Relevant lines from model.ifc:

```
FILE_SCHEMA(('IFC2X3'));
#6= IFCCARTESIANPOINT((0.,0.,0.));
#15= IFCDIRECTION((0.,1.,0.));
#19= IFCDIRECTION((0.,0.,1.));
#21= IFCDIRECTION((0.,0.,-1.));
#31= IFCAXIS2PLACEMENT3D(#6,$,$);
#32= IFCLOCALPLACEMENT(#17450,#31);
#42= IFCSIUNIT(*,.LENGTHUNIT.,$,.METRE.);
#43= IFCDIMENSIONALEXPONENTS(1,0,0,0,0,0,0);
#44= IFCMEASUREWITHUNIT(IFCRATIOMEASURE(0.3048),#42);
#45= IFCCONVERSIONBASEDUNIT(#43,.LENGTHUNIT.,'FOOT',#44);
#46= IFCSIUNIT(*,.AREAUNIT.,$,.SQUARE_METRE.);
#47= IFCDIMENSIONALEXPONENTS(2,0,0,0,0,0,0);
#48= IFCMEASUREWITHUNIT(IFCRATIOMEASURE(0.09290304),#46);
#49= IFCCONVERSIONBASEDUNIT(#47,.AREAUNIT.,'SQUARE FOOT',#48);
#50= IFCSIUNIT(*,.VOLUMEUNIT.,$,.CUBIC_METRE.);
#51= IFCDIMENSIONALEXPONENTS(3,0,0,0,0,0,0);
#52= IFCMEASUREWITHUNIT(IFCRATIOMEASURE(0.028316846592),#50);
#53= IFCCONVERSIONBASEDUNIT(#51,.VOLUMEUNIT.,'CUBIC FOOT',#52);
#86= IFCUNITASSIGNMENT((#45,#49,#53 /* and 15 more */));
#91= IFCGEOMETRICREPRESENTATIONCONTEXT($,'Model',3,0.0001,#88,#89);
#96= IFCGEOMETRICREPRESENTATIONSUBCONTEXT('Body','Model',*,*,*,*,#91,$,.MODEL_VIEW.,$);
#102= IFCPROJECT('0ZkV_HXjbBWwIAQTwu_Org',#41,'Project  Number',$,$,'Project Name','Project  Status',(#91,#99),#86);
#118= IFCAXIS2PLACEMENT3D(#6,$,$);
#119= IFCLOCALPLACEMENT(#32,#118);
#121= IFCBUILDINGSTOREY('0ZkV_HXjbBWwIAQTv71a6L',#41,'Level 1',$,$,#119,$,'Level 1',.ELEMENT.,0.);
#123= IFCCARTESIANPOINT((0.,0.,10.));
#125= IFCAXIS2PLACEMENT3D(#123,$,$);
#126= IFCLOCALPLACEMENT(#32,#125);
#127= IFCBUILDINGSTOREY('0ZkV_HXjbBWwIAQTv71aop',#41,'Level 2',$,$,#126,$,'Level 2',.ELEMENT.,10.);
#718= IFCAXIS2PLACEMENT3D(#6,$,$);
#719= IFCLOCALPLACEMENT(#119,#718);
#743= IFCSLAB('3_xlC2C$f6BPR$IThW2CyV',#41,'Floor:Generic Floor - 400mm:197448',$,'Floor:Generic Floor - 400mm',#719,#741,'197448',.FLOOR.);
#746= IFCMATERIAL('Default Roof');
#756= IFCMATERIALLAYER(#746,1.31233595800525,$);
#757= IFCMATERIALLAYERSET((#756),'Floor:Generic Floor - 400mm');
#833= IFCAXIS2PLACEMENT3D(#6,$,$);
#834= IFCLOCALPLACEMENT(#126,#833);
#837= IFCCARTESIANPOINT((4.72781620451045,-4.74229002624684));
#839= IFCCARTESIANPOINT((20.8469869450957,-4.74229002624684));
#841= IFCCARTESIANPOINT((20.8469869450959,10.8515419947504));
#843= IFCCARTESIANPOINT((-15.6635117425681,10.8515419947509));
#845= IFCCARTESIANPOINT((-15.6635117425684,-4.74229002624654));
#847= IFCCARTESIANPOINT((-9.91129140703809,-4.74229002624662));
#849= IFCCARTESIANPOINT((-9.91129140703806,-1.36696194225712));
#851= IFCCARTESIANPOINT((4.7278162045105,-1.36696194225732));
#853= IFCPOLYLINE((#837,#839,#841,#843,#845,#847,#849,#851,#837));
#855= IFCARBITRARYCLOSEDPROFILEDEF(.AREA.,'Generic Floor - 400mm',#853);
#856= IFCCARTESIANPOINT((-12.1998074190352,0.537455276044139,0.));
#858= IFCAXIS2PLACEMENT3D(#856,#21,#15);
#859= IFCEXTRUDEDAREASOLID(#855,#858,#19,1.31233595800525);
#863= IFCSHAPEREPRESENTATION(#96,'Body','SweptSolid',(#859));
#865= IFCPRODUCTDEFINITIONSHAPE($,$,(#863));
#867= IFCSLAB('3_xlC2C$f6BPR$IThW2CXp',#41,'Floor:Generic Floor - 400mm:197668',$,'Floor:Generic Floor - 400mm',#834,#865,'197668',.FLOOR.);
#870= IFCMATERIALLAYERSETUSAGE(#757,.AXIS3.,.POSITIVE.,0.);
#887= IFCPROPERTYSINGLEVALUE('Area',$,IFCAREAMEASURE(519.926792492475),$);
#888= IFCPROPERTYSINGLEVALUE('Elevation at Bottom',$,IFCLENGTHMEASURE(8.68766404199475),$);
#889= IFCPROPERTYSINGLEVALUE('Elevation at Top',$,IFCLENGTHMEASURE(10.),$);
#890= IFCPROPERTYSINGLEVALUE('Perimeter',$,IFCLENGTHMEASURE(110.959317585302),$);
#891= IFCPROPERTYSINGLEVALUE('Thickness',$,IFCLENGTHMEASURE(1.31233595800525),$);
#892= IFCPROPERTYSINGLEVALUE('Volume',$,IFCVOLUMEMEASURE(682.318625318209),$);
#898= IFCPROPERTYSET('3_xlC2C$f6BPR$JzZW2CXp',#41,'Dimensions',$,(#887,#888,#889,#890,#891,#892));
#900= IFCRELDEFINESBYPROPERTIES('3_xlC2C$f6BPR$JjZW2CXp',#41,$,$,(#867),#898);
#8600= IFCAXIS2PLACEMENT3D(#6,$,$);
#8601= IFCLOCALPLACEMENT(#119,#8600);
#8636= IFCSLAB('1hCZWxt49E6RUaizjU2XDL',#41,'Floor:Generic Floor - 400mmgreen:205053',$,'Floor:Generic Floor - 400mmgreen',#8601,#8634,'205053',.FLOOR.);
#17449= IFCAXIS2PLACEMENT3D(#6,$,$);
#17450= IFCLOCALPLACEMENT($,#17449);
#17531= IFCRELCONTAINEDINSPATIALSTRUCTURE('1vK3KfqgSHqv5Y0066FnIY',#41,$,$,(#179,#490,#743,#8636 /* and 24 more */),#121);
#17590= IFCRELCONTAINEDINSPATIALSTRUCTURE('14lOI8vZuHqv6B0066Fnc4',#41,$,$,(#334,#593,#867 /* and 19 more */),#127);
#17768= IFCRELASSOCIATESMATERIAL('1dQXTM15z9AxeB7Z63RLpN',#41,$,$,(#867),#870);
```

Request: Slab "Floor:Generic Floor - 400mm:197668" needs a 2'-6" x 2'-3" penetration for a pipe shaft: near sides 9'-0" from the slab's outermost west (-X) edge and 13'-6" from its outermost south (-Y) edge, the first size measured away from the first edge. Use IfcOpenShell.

```python
import numpy as np
import ifcopenshell
import ifcopenshell.api.feature
import ifcopenshell.api.geometry
import ifcopenshell.api.pset
import ifcopenshell.api.root
import ifcopenshell.geom
import ifcopenshell.util.element
import ifcopenshell.util.placement
import ifcopenshell.util.representation
import ifcopenshell.util.shape
import ifcopenshell.util.unit

model = ifcopenshell.open("model.ifc")
unit_scale = ifcopenshell.util.unit.calculate_unit_scale(model)
area_scale = ifcopenshell.util.unit.calculate_unit_scale(model, "AREAUNIT")
volume_scale = ifcopenshell.util.unit.calculate_unit_scale(model, "VOLUMEUNIT")
settings = ifcopenshell.geom.settings()


def volume(element):
    """Net volume in cubic metres, openings subtracted."""
    shape = ifcopenshell.geom.create_shape(settings, element)
    return ifcopenshell.util.shape.get_volume(shape.geometry)


slab = model.by_id(867)
before = volume(slab)

# Extent in the slab's own axes, in metres. The edges named are its -X and -Y sides.
slab_shape = ifcopenshell.geom.create_shape(settings, slab)
vertices = ifcopenshell.util.shape.get_vertices(slab_shape.geometry)
x_min, y_min, bottom = vertices.min(axis=0)
top = vertices[:, 2].max()

opening = ifcopenshell.api.root.create_entity(model, ifc_class="IfcOpeningElement", name="Pipe shaft opening")
context = ifcopenshell.util.representation.get_context(model, "Model", "Body", "MODEL_VIEW")
width, depth = 0.762, 0.6858
outline = [(0.0, 0.0), (width, 0.0), (width, depth), (0.0, depth), (0.0, 0.0)]
# Overshoot both faces by 50 mm so the cut is clean.
shape = ifcopenshell.api.geometry.add_slab_representation(
    model, context=context, depth=top - bottom + 0.1, polyline=outline
)
ifcopenshell.api.geometry.assign_representation(model, product=opening, representation=shape)

matrix = ifcopenshell.util.placement.get_local_placement(slab.ObjectPlacement)
matrix[:, 3] = matrix @ np.append(np.array([x_min + 2.7432, y_min + 4.1148, bottom - 0.05]) / unit_scale, 1.0)
ifcopenshell.api.geometry.edit_object_placement(model, product=opening, matrix=matrix, is_si=False)
ifcopenshell.api.feature.add_feature(model, feature=opening, element=slab)

after = volume(slab)

# Update the slab's stored quantities.
pset = model.by_id(ifcopenshell.util.element.get_pset(slab, "Dimensions", should_inherit=False)["id"])
ifcopenshell.api.pset.edit_pset(model, pset=pset, properties={
    "Area": model.create_entity("IfcAreaMeasure", after / (top - bottom) / area_scale),
    "Volume": model.create_entity("IfcVolumeMeasure", after / volume_scale),
})

print(f"slab volume {before:.3f} -> {after:.3f} m3")

model.write("model_updated.ifc")
```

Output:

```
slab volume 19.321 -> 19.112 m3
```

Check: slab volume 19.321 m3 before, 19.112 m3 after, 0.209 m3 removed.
